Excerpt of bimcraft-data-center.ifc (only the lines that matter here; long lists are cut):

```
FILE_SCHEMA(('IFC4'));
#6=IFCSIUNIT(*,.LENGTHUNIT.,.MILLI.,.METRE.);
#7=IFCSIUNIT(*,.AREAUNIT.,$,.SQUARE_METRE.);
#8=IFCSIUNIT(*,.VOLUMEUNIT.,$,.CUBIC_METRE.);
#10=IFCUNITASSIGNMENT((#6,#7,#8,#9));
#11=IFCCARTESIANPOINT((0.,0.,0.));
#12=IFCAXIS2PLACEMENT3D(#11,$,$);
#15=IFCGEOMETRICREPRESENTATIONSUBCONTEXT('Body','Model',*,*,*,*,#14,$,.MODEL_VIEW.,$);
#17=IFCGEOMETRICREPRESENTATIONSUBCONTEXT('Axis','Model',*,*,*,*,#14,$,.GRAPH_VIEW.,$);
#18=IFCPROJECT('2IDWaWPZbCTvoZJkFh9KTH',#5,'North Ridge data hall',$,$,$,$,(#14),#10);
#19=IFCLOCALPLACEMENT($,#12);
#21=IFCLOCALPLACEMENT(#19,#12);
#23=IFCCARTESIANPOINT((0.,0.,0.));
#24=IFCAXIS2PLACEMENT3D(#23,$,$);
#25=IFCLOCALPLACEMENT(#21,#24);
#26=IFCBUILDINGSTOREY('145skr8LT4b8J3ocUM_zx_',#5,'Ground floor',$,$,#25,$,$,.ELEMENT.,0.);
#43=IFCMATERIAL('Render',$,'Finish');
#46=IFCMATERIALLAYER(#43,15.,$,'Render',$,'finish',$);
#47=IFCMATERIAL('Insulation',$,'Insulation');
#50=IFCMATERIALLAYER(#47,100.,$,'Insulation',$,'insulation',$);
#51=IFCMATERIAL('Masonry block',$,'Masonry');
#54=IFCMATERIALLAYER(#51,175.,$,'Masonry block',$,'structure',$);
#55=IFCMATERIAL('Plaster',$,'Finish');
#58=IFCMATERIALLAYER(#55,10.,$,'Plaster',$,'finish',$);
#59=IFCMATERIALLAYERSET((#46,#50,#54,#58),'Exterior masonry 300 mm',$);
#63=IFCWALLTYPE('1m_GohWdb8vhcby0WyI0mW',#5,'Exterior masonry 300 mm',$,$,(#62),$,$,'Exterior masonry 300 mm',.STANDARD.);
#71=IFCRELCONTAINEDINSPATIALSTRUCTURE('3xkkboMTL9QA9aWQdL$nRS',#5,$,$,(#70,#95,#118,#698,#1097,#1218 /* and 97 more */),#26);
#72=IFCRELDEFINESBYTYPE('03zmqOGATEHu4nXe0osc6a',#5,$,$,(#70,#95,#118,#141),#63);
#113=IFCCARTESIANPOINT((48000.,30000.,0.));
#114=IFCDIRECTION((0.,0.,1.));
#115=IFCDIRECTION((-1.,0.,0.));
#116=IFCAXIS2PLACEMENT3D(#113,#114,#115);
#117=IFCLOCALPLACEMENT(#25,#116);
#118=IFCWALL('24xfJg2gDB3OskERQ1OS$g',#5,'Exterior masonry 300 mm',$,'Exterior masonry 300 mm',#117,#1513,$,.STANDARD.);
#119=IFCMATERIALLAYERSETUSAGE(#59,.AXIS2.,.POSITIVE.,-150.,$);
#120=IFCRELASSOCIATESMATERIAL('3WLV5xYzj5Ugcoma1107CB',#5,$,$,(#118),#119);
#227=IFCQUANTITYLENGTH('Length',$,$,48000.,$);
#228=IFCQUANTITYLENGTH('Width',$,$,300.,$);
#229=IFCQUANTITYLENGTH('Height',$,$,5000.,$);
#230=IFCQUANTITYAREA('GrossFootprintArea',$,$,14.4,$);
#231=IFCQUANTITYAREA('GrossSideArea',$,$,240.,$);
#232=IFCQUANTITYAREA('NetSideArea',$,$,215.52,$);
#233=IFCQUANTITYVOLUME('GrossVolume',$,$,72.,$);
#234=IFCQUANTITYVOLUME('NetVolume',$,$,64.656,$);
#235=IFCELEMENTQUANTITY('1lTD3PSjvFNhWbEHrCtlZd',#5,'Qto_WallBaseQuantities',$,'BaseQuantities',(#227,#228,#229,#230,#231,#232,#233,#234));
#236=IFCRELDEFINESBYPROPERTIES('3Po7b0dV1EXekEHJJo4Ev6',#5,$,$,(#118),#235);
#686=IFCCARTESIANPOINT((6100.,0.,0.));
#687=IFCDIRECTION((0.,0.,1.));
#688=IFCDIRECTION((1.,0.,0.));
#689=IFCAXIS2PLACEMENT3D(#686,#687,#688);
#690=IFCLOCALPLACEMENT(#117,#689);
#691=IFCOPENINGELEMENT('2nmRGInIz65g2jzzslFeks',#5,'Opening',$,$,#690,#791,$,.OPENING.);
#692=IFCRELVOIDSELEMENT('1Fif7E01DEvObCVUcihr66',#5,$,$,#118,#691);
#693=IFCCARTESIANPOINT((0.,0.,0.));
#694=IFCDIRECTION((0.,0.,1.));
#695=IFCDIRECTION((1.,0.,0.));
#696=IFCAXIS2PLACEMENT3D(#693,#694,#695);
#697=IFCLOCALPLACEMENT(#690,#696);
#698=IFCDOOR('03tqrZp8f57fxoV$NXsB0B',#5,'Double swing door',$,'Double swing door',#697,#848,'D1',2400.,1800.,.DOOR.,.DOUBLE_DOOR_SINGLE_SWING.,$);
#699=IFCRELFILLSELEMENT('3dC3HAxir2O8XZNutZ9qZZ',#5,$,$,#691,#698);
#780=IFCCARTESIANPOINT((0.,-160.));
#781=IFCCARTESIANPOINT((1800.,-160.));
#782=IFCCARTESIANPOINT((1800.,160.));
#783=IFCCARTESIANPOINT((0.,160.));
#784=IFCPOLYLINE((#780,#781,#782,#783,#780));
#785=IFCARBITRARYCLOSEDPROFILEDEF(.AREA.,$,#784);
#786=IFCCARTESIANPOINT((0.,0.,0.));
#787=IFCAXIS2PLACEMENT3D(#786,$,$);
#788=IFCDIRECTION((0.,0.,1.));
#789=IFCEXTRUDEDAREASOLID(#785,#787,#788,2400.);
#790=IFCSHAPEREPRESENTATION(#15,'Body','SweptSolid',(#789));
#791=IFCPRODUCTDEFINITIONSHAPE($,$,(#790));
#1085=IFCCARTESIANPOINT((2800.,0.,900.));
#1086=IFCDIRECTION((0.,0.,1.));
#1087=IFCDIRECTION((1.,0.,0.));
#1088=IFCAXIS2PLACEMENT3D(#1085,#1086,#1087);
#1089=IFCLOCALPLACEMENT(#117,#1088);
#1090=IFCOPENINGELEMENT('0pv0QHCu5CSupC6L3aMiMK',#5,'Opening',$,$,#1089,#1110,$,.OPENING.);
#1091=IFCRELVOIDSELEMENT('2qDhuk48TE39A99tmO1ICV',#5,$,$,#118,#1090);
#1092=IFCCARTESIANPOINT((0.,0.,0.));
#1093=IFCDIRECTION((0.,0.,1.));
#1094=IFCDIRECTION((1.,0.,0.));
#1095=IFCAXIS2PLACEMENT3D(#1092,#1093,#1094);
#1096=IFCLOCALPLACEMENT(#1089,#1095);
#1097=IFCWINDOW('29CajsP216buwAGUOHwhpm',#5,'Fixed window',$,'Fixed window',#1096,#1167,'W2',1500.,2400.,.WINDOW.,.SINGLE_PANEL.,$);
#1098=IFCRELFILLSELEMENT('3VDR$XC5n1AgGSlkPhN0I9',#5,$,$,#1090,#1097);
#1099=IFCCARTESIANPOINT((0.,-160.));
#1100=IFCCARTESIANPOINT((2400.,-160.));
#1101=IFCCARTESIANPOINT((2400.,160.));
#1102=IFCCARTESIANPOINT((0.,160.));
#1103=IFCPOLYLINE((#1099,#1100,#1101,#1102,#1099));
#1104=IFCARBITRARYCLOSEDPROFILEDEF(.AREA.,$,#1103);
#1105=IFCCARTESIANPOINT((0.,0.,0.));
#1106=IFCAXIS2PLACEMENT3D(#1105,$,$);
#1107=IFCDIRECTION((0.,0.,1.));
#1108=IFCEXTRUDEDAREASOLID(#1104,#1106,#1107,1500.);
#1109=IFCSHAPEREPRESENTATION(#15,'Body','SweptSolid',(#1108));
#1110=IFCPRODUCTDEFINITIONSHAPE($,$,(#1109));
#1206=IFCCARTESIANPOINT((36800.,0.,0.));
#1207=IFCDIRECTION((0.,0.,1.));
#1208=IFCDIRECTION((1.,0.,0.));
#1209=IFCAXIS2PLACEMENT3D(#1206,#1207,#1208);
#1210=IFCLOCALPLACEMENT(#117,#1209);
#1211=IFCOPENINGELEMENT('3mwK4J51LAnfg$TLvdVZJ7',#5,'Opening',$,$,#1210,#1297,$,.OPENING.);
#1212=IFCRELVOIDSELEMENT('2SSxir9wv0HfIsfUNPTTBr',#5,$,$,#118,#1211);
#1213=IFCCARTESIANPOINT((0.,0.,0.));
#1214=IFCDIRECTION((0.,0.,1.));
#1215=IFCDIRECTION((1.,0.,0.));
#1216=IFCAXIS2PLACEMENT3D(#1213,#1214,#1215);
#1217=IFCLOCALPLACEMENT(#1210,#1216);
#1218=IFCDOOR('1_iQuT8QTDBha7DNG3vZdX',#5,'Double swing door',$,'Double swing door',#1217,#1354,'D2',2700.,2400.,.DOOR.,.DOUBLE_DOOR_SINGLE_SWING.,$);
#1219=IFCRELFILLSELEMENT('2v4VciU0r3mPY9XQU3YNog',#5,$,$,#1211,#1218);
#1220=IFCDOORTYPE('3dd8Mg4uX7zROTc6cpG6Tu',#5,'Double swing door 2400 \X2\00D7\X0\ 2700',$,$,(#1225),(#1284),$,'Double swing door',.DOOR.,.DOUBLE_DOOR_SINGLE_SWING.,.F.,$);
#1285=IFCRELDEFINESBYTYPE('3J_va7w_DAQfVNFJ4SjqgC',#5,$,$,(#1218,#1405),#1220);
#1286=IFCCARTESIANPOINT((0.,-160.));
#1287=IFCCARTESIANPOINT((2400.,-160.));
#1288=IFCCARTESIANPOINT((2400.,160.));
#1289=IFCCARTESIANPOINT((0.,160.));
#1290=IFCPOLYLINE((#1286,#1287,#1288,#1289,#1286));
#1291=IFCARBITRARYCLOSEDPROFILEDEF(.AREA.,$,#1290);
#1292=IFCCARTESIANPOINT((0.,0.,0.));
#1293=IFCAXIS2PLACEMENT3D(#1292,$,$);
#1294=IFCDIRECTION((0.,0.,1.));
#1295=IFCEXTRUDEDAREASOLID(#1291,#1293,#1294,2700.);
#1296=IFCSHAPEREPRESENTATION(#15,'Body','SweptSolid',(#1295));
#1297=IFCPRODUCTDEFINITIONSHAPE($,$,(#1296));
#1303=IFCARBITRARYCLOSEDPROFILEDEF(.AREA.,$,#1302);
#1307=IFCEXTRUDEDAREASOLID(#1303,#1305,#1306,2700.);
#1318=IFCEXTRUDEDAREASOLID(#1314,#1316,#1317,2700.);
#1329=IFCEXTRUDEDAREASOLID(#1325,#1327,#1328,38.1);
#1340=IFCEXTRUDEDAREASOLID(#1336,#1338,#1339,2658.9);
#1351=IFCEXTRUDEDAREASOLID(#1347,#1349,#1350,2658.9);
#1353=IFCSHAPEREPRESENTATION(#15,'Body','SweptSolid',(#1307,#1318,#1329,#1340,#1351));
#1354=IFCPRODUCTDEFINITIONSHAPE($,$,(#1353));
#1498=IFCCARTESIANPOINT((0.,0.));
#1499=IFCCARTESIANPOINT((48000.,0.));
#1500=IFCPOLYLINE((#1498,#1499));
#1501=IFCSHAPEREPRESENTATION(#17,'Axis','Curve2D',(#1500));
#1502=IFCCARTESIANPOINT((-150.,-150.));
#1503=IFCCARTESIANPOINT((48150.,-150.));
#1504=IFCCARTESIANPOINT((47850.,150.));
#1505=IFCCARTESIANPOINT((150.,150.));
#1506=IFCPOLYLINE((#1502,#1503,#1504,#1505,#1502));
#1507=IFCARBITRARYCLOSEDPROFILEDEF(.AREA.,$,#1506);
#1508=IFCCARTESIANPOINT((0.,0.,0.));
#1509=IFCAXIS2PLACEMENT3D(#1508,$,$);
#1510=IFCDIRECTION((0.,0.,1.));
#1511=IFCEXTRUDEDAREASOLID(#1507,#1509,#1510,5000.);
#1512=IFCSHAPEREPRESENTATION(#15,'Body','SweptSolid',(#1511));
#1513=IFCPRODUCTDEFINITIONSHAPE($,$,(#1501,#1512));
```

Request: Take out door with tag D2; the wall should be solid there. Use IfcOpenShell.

```python
import ifcopenshell
import ifcopenshell.api.feature
import ifcopenshell.api.pset
import ifcopenshell.api.root
import ifcopenshell.geom
import ifcopenshell.util.element
import ifcopenshell.util.shape
import ifcopenshell.util.unit

model = ifcopenshell.open("bimcraft-data-center.ifc")
area_scale = ifcopenshell.util.unit.calculate_unit_scale(model, "AREAUNIT")
volume_scale = ifcopenshell.util.unit.calculate_unit_scale(model, "VOLUMEUNIT")
settings = ifcopenshell.geom.settings()


def volume(element):
    """Net volume in cubic metres, openings subtracted."""
    shape = ifcopenshell.geom.create_shape(settings, element)
    return ifcopenshell.util.shape.get_volume(shape.geometry)


door = model.by_guid("1_iQuT8QTDBha7DNG3vZdX")
opening = door.FillsVoids[0].RelatingOpeningElement
wall = opening.VoidsElements[0].RelatingBuildingElement
before = volume(wall)

ifcopenshell.api.root.remove_product(model, product=door)
ifcopenshell.api.feature.remove_feature(model, feature=opening)

after = volume(wall)
thickness = 0.3  # wall thickness in metres

# Update the wall's stored quantities.
qto = model.by_id(ifcopenshell.util.element.get_pset(wall, "Qto_WallBaseQuantities", should_inherit=False)["id"])
ifcopenshell.api.pset.edit_qto(model, qto=qto, properties={
    "NetSideArea": after / thickness / area_scale,
    "NetVolume": after / volume_scale,
})

print(f"wall volume {before:.3f} -> {after:.3f} m3")

model.write("bimcraft-data-center-out.ifc")
```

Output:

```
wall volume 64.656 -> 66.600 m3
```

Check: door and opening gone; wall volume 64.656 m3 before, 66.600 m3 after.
